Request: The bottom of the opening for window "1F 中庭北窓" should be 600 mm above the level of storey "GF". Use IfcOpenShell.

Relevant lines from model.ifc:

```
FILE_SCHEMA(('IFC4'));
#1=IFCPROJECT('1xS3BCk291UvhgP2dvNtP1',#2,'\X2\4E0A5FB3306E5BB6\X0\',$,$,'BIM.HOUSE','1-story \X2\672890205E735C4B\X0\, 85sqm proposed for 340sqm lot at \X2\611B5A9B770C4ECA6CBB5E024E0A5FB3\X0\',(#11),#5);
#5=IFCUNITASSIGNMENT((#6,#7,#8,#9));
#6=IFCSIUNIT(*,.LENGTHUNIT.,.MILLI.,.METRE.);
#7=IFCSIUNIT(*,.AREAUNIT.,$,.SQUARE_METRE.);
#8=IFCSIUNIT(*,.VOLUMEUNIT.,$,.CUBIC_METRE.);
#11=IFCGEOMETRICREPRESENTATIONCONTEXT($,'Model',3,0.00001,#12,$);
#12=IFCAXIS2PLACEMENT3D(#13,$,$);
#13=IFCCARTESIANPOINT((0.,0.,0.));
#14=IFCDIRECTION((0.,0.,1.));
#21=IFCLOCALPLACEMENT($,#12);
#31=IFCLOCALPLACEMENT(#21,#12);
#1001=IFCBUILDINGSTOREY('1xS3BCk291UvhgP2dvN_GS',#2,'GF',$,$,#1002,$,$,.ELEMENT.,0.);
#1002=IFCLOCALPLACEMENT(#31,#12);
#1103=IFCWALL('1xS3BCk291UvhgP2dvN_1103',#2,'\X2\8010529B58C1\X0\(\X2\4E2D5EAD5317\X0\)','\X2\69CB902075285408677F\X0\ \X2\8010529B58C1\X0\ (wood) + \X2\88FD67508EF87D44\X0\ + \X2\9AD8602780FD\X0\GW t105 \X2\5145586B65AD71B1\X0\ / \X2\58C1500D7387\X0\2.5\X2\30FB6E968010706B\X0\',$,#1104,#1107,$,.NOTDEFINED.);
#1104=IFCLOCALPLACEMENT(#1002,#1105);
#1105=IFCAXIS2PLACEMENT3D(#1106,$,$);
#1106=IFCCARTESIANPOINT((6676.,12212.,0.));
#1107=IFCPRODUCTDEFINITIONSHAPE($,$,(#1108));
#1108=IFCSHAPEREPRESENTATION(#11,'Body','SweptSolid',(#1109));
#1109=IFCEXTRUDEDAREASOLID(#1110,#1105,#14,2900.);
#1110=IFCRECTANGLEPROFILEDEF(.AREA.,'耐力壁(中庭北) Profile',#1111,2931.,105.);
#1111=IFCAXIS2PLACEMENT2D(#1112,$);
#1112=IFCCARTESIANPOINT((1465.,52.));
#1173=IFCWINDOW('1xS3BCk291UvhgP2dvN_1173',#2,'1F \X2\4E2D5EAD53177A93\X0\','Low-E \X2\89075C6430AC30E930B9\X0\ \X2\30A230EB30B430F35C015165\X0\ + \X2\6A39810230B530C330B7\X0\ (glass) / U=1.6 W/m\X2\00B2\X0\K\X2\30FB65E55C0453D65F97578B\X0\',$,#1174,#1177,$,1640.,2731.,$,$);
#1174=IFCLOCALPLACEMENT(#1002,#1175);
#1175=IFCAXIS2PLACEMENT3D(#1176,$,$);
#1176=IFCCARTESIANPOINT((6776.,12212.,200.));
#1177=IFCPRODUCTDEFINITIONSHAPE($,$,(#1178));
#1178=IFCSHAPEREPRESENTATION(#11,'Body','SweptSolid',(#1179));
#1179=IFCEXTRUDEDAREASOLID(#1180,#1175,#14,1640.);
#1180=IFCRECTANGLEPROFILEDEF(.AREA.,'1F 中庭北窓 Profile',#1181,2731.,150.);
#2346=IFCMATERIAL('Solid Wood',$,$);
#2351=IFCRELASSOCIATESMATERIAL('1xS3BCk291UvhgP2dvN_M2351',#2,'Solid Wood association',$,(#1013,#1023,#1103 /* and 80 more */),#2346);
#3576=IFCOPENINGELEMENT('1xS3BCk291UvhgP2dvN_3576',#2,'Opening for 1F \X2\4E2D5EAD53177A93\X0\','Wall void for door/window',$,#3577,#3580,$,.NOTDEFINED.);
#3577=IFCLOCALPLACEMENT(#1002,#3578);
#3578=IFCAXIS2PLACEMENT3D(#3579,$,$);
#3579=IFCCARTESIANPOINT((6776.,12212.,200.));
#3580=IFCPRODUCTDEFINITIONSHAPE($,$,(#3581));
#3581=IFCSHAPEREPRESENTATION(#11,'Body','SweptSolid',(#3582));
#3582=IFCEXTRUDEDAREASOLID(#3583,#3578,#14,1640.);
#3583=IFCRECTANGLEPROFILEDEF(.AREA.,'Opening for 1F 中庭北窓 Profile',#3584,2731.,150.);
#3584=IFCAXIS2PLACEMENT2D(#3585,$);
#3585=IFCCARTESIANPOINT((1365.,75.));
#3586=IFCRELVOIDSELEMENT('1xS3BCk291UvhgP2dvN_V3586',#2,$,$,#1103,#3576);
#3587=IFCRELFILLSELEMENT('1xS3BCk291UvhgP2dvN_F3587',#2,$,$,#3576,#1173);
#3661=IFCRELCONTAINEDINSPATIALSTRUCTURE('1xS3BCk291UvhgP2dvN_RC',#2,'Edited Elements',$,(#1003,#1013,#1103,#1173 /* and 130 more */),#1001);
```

```python
import numpy as np
import ifcopenshell
import ifcopenshell.api.geometry
import ifcopenshell.geom
import ifcopenshell.util.element
import ifcopenshell.util.placement
import ifcopenshell.util.shape
import ifcopenshell.util.unit

model = ifcopenshell.open("model.ifc")
unit_scale = ifcopenshell.util.unit.calculate_unit_scale(model)

window = model.by_guid("1xS3BCk291UvhgP2dvN_1173")
opening = window.FillsVoids[0].RelatingOpeningElement
storey = ifcopenshell.util.element.get_container(window, ifc_class="IfcBuildingStorey")
level = ifcopenshell.util.placement.get_local_placement(storey.ObjectPlacement)[2, 3]

# The opening's origin need not be at the sill, so measure its lowest point.
shape = ifcopenshell.geom.create_shape(ifcopenshell.geom.settings(), opening)
bottom = ifcopenshell.util.shape.get_shape_bottom_elevation(shape, shape.geometry) / unit_scale
dz = level + 600.0 - bottom

shift = np.array([0.0, 0.0, dz])
# The window is not placed relative to its opening, so move both.
for product in (opening, window):
    matrix = ifcopenshell.util.placement.get_local_placement(product.ObjectPlacement)
    matrix[:3, 3] += shift
    ifcopenshell.api.geometry.edit_object_placement(model, product=product, matrix=matrix, is_si=False)

print(f"moved by {dz * unit_scale:+.3f} m")

model.write("model_rev.ifc")
```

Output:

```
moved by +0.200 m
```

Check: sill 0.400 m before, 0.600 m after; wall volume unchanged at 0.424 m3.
